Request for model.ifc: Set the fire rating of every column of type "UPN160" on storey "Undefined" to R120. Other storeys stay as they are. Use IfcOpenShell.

First a look at what the model holds.

```python
import ifcopenshell
import ifcopenshell.util.element

model = ifcopenshell.open("model.ifc")
print(model.schema)
storey = next(s for s in model.by_type("IfcBuildingStorey") if s.Name == "Undefined")
columns = [e for e in ifcopenshell.util.element.get_decomposition(storey) if e.is_a("IfcColumn")]
seen = {}
for e in columns:
    element_type = ifcopenshell.util.element.get_type(e)
    key = (element_type.Name if element_type != e and element_type else None, ifcopenshell.util.element.get_pset(e, "Pset_ColumnCommon", "FireRating"))
    seen[key] = seen.get(key, 0) + 1
for (name, value), count in sorted(seen.items(), key=str):
    print(count, "x", name, "|", value)
```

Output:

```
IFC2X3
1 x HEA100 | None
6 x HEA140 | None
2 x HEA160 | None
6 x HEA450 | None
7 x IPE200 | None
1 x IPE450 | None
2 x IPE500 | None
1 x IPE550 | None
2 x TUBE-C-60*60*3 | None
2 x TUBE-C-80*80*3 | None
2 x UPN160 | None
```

```python
import ifcopenshell
import ifcopenshell.api.pset
import ifcopenshell.util.element

model = ifcopenshell.open("model.ifc")

storey = next(s for s in model.by_type("IfcBuildingStorey") if s.Name == "Undefined")
columns = [e for e in ifcopenshell.util.element.get_decomposition(storey) if e.is_a("IfcColumn")]

count = 0
for e in columns:
    element_type = ifcopenshell.util.element.get_type(e)
    if element_type in (None, e) or element_type.Name != "UPN160":
        continue
    # add_pset returns the element's existing set when there is one.
    pset = ifcopenshell.api.pset.add_pset(model, product=e, name="Pset_ColumnCommon")
    ifcopenshell.api.pset.edit_pset(model, pset=pset, properties={"FireRating": "R120"})
    count += 1

print(count, "columns updated")

model.write("model_v2.ifc")
```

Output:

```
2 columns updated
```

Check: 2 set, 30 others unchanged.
